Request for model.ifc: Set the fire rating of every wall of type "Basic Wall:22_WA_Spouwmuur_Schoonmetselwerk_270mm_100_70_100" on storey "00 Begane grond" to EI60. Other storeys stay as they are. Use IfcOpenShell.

First a look at what the model holds.

```python
import ifcopenshell
import ifcopenshell.util.element

model = ifcopenshell.open("model.ifc")
print(model.schema)
storey = next(s for s in model.by_type("IfcBuildingStorey") if s.Name == "00 Begane grond")
walls = [e for e in ifcopenshell.util.element.get_decomposition(storey) if e.is_a("IfcWall")]
seen = {}
for e in walls:
    element_type = ifcopenshell.util.element.get_type(e)
    key = (element_type.Name if element_type != e and element_type else None, ifcopenshell.util.element.get_pset(e, "Pset_WallCommon", "FireRating"))
    seen[key] = seen.get(key, 0) + 1
for (name, value), count in sorted(seen.items(), key=str):
    print(count, "x", name, "|", value)
```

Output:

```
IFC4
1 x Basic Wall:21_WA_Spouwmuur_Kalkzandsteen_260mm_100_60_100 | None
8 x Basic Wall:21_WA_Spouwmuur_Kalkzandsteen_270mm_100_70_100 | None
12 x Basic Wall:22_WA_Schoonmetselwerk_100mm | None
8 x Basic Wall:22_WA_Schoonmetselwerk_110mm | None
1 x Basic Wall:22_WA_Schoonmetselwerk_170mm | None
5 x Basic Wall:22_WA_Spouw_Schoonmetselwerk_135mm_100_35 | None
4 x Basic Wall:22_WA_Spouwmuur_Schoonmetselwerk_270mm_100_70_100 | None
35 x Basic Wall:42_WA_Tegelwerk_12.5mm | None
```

```python
import ifcopenshell
import ifcopenshell.api.pset
import ifcopenshell.util.element

model = ifcopenshell.open("model.ifc")

storey = next(s for s in model.by_type("IfcBuildingStorey") if s.Name == "00 Begane grond")
walls = [e for e in ifcopenshell.util.element.get_decomposition(storey) if e.is_a("IfcWall")]

count = 0
for e in walls:
    element_type = ifcopenshell.util.element.get_type(e)
    if element_type in (None, e) or element_type.Name != "Basic Wall:22_WA_Spouwmuur_Schoonmetselwerk_270mm_100_70_100":
        continue
    # add_pset returns the element's existing set when there is one.
    pset = ifcopenshell.api.pset.add_pset(model, product=e, name="Pset_WallCommon")
    ifcopenshell.api.pset.edit_pset(model, pset=pset, properties={"FireRating": "EI60"})
    count += 1

print(count, "walls updated")

model.write("model-out.ifc")
```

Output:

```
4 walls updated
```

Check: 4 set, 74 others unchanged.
